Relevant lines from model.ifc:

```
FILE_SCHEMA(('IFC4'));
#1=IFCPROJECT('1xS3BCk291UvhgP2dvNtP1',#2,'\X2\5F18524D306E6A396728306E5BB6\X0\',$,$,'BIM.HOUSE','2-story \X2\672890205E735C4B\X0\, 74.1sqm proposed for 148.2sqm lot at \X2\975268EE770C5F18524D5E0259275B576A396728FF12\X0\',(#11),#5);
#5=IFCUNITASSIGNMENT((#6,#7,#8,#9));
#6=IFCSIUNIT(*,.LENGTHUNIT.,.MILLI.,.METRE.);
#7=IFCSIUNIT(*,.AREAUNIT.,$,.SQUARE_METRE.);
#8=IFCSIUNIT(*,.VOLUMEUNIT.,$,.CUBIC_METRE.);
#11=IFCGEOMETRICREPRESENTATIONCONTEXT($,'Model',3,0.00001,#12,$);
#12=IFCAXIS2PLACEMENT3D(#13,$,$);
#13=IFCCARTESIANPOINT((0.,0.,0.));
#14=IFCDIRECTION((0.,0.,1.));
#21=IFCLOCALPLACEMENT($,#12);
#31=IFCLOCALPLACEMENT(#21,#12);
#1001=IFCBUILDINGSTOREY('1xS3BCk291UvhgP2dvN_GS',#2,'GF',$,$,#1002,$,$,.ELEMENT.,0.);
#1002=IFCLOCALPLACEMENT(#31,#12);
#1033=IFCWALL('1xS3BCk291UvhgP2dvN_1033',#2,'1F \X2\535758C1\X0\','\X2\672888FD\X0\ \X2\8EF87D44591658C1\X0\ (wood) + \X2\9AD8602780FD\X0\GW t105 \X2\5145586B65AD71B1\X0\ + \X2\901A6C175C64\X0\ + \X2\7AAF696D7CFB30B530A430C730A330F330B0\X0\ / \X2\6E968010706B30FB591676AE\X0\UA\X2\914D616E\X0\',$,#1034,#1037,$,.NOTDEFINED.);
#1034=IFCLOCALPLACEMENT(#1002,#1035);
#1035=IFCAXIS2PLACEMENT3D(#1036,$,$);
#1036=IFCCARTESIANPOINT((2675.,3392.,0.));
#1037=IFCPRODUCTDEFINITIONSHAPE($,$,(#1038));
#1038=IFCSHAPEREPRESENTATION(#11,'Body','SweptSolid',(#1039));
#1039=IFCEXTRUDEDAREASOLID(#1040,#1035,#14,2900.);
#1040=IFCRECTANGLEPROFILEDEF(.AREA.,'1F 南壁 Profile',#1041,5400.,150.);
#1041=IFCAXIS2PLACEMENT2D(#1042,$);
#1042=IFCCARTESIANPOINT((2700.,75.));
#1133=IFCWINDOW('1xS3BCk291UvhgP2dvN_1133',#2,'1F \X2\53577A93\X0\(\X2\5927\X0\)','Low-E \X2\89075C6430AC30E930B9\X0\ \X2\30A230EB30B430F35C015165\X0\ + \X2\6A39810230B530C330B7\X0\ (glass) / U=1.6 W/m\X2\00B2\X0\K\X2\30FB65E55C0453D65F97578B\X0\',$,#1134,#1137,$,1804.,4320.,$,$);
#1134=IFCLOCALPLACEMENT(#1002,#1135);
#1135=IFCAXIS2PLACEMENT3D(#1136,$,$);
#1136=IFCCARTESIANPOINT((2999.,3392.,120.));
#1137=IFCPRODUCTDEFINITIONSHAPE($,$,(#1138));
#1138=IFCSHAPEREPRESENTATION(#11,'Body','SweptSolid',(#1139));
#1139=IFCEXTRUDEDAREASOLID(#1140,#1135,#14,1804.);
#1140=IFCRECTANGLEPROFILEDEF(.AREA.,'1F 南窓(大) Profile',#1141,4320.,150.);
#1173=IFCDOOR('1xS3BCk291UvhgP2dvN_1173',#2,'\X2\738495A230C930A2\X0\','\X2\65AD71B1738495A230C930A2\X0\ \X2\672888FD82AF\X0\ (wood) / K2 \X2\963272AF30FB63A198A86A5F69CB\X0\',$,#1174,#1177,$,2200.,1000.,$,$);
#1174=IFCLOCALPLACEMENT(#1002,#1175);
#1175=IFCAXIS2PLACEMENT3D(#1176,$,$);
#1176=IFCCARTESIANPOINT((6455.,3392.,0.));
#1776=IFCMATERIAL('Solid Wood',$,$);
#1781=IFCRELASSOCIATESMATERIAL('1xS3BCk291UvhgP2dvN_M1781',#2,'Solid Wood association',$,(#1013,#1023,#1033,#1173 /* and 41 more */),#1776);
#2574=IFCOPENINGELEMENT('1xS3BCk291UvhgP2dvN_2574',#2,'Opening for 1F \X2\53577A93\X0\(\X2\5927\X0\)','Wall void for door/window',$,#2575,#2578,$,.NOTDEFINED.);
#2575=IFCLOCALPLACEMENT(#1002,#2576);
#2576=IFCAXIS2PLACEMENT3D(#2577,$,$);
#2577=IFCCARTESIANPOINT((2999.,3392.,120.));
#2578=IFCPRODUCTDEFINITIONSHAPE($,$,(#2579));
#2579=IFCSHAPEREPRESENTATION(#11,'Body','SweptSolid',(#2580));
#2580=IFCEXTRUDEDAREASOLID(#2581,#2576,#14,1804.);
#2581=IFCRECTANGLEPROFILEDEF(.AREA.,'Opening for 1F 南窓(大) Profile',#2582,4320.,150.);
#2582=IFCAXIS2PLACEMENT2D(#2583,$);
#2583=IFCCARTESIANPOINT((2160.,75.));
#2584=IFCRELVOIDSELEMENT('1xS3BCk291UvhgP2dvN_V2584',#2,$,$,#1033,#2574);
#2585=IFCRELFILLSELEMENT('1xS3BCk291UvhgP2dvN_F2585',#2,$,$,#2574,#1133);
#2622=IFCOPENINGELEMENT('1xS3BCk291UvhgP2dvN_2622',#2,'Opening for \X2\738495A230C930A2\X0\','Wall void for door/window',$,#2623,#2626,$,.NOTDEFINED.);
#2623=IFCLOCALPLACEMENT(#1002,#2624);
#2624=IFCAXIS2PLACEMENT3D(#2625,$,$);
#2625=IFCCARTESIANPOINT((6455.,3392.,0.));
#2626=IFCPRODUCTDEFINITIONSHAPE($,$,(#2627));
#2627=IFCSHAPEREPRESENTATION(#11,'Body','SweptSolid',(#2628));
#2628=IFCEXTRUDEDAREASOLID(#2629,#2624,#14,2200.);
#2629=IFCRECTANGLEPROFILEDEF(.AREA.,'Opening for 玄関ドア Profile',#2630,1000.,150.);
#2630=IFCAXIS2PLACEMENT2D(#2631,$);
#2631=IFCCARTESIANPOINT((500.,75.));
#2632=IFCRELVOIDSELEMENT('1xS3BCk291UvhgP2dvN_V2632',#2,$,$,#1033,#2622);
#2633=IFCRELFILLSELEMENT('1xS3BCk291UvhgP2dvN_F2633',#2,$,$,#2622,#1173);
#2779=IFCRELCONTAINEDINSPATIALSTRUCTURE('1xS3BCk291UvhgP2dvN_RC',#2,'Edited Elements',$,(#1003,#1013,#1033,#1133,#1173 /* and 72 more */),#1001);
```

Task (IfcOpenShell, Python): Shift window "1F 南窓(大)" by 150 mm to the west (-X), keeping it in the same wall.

```python
import ifcopenshell
import ifcopenshell.api.geometry
import ifcopenshell.util.placement
import ifcopenshell.util.unit

model = ifcopenshell.open("model.ifc")
unit_scale = ifcopenshell.util.unit.calculate_unit_scale(model)

window = model.by_guid("1xS3BCk291UvhgP2dvN_1133")
opening = window.FillsVoids[0].RelatingOpeningElement
wall = opening.VoidsElements[0].RelatingBuildingElement

wall_matrix = ifcopenshell.util.placement.get_local_placement(wall.ObjectPlacement)
shift = wall_matrix[:3, 0] * -0.15 / unit_scale
before = ifcopenshell.util.placement.get_local_placement(window.ObjectPlacement)[:3, 3].copy()

# The window is not placed relative to its opening, so move both.
for product in (opening, window):
    matrix = ifcopenshell.util.placement.get_local_placement(product.ObjectPlacement)
    matrix[:3, 3] += shift
    ifcopenshell.api.geometry.edit_object_placement(model, product=product, matrix=matrix, is_si=False)

after = ifcopenshell.util.placement.get_local_placement(window.ObjectPlacement)[:3, 3]
print("window moved by", (after - before).round(3) + 0.0)

model.write("model_edited.ifc")
```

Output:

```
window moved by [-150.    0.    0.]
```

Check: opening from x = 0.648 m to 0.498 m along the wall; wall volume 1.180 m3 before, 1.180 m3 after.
